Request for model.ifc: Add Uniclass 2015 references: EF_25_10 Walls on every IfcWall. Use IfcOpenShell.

First a look at what the model holds.

```python
import ifcopenshell

model = ifcopenshell.open("model.ifc")
print(model.schema)
print("classifications:", [c.Name for c in model.by_type("IfcClassification")])
for ifc_class in ("IfcDoor", "IfcRoof", "IfcStair", "IfcWall", "IfcWindow"):
    print(ifc_class, len(model.by_type(ifc_class)))
```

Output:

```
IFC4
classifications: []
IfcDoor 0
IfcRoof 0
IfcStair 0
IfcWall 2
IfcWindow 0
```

```python
import ifcopenshell
import ifcopenshell.api.classification

model = ifcopenshell.open("model.ifc")

system = ifcopenshell.api.classification.add_classification(model, classification="Uniclass 2015")

codes = {
    "IfcWall": ("EF_25_10", "Walls"),
}
for ifc_class, (code, name) in codes.items():
    products = model.by_type(ifc_class)
    ifcopenshell.api.classification.add_reference(
        model, products=products, classification=system, identification=code, name=name
    )
    print(code, len(products))

model.write("model_rev.ifc")
```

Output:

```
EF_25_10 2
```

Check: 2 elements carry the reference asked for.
